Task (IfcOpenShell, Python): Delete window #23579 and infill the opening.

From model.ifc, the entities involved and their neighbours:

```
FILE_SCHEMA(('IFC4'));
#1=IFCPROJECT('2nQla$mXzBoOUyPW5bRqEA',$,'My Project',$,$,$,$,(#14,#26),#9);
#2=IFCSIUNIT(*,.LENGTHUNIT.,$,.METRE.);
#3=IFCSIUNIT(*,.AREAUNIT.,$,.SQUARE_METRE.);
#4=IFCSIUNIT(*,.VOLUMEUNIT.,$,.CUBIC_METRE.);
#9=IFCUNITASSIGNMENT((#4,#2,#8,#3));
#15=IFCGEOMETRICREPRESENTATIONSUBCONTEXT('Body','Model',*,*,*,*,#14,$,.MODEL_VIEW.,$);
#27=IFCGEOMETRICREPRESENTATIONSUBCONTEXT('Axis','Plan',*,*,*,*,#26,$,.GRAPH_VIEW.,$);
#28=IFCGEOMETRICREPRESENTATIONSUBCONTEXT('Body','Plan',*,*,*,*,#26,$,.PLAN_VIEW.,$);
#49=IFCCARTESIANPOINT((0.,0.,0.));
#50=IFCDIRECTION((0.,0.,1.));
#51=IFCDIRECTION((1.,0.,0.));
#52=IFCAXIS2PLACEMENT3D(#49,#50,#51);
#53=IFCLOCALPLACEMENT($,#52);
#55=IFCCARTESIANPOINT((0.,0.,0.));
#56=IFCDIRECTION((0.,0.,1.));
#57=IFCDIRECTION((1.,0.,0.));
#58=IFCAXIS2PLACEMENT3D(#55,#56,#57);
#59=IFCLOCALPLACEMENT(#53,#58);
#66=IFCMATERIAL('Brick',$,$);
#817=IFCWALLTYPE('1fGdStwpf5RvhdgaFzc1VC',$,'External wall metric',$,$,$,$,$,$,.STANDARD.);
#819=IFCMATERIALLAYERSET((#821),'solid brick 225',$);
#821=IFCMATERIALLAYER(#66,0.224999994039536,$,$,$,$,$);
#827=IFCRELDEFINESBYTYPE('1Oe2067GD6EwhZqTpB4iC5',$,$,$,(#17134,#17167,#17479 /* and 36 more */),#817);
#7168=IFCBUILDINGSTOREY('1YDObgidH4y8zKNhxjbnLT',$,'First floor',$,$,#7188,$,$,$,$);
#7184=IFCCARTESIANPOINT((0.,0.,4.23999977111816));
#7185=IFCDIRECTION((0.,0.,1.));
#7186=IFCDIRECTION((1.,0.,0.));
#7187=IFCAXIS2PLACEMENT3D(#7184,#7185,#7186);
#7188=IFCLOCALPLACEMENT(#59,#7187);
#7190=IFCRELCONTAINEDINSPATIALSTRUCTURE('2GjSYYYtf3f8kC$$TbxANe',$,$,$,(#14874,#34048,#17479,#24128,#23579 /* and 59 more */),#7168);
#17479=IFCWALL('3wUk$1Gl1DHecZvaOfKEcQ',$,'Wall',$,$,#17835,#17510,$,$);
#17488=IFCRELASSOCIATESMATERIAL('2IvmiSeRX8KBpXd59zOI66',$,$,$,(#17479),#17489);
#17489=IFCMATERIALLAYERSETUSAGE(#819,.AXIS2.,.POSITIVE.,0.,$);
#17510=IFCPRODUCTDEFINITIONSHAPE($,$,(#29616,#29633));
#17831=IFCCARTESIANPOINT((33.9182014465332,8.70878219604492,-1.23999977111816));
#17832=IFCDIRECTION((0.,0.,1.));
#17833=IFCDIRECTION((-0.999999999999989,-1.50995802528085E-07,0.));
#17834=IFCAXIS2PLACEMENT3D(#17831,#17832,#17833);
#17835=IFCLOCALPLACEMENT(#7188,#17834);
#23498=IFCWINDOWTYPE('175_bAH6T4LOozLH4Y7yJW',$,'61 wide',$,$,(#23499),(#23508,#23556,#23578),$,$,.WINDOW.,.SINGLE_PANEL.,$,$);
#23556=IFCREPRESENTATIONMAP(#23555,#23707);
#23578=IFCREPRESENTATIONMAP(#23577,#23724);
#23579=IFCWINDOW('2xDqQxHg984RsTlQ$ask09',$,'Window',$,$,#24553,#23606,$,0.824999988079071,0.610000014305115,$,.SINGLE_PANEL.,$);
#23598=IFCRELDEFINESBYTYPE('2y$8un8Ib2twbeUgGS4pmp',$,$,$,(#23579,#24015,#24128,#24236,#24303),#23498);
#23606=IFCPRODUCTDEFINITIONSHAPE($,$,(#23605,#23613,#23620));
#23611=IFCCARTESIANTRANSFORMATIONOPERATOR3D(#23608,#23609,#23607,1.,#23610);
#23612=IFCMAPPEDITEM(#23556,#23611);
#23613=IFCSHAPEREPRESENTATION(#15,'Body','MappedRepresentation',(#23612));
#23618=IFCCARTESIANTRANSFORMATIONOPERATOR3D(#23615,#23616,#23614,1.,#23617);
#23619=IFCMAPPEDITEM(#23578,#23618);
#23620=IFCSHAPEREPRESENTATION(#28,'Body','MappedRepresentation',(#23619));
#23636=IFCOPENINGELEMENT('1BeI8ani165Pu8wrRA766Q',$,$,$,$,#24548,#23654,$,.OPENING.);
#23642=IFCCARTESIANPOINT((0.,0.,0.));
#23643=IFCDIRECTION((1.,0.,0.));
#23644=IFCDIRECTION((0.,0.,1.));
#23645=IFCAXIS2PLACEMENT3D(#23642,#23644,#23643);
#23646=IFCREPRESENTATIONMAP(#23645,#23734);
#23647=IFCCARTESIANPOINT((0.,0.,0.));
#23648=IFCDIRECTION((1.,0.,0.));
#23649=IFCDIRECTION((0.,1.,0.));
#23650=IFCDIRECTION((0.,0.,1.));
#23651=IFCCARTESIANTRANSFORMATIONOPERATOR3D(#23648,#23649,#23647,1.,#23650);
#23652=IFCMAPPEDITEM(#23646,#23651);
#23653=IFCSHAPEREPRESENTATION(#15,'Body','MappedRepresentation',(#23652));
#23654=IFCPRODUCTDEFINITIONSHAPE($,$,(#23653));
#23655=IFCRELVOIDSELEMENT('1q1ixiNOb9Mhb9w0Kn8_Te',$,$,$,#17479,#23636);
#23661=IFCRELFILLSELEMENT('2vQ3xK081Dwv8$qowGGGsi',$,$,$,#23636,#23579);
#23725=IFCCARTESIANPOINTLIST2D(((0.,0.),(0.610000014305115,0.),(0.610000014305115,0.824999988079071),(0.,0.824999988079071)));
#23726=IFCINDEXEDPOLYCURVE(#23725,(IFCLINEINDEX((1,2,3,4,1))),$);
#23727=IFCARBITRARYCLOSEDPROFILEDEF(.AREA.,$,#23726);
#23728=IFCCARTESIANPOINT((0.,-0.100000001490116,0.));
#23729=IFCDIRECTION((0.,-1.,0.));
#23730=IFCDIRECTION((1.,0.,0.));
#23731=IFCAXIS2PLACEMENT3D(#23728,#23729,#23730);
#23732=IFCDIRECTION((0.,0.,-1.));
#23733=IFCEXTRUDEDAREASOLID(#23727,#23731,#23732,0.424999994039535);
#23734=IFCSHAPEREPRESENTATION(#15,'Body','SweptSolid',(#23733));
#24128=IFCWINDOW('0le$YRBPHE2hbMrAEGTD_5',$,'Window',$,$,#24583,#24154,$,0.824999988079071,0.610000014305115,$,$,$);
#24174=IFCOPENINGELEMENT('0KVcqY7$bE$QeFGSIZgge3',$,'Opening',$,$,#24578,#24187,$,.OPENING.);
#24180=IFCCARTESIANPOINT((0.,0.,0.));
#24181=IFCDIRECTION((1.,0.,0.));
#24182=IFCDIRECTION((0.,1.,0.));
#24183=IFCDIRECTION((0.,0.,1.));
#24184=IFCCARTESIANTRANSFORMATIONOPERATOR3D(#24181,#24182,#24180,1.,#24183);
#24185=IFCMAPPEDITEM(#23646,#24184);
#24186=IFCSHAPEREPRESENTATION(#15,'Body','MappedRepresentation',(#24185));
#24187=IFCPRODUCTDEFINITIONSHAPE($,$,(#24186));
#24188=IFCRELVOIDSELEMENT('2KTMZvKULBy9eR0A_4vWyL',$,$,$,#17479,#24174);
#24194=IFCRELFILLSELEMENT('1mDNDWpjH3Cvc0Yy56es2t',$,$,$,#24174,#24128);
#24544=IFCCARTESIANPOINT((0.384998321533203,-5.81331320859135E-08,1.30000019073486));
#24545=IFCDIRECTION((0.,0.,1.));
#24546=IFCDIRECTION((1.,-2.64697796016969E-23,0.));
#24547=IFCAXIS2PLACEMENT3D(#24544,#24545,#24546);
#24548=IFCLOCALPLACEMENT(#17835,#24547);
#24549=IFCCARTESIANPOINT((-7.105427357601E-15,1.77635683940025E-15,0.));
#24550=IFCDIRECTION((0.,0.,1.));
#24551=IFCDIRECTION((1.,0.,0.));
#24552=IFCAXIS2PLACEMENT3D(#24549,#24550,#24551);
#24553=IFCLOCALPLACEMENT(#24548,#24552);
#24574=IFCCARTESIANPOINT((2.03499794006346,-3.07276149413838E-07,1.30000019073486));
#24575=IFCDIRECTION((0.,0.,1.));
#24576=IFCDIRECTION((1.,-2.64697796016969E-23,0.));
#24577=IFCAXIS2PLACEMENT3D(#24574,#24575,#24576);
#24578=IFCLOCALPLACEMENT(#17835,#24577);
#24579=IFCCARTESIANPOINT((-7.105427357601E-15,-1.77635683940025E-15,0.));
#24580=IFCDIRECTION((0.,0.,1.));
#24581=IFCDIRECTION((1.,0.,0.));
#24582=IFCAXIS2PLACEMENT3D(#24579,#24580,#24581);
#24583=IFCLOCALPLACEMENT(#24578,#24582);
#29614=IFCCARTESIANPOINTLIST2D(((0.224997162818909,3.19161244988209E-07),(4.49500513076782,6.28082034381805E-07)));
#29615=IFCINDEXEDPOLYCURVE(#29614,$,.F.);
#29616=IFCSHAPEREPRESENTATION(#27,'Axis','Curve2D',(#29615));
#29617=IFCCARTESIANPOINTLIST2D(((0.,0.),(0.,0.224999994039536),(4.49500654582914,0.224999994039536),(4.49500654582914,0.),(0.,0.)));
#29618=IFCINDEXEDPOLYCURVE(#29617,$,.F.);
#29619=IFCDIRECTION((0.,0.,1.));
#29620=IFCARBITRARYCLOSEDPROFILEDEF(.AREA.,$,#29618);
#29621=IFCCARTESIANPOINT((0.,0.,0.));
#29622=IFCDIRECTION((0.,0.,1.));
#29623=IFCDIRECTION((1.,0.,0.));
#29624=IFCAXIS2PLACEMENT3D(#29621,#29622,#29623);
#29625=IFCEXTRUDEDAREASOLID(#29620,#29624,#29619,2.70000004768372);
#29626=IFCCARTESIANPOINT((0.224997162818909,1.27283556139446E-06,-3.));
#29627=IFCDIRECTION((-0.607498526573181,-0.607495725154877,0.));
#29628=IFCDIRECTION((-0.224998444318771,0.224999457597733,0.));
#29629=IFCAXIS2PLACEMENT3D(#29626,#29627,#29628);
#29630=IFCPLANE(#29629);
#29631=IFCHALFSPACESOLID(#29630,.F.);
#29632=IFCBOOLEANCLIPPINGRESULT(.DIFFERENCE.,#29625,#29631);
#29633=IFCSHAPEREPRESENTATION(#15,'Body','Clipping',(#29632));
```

```python
import ifcopenshell
import ifcopenshell.api.feature
import ifcopenshell.api.root
import ifcopenshell.geom
import ifcopenshell.util.shape

model = ifcopenshell.open("model.ifc")
settings = ifcopenshell.geom.settings()


def volume(element):
    """Net volume in cubic metres, openings subtracted."""
    shape = ifcopenshell.geom.create_shape(settings, element)
    return ifcopenshell.util.shape.get_volume(shape.geometry)


window = model.by_guid("2xDqQxHg984RsTlQ$ask09")
opening = window.FillsVoids[0].RelatingOpeningElement
wall = opening.VoidsElements[0].RelatingBuildingElement
before = volume(wall)

ifcopenshell.api.root.remove_product(model, product=window)
ifcopenshell.api.feature.remove_feature(model, feature=opening)

after = volume(wall)

print(f"wall volume {before:.3f} -> {after:.3f} m3")

model.write("model_rev.ifc")
```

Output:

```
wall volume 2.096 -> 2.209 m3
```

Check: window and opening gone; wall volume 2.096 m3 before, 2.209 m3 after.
